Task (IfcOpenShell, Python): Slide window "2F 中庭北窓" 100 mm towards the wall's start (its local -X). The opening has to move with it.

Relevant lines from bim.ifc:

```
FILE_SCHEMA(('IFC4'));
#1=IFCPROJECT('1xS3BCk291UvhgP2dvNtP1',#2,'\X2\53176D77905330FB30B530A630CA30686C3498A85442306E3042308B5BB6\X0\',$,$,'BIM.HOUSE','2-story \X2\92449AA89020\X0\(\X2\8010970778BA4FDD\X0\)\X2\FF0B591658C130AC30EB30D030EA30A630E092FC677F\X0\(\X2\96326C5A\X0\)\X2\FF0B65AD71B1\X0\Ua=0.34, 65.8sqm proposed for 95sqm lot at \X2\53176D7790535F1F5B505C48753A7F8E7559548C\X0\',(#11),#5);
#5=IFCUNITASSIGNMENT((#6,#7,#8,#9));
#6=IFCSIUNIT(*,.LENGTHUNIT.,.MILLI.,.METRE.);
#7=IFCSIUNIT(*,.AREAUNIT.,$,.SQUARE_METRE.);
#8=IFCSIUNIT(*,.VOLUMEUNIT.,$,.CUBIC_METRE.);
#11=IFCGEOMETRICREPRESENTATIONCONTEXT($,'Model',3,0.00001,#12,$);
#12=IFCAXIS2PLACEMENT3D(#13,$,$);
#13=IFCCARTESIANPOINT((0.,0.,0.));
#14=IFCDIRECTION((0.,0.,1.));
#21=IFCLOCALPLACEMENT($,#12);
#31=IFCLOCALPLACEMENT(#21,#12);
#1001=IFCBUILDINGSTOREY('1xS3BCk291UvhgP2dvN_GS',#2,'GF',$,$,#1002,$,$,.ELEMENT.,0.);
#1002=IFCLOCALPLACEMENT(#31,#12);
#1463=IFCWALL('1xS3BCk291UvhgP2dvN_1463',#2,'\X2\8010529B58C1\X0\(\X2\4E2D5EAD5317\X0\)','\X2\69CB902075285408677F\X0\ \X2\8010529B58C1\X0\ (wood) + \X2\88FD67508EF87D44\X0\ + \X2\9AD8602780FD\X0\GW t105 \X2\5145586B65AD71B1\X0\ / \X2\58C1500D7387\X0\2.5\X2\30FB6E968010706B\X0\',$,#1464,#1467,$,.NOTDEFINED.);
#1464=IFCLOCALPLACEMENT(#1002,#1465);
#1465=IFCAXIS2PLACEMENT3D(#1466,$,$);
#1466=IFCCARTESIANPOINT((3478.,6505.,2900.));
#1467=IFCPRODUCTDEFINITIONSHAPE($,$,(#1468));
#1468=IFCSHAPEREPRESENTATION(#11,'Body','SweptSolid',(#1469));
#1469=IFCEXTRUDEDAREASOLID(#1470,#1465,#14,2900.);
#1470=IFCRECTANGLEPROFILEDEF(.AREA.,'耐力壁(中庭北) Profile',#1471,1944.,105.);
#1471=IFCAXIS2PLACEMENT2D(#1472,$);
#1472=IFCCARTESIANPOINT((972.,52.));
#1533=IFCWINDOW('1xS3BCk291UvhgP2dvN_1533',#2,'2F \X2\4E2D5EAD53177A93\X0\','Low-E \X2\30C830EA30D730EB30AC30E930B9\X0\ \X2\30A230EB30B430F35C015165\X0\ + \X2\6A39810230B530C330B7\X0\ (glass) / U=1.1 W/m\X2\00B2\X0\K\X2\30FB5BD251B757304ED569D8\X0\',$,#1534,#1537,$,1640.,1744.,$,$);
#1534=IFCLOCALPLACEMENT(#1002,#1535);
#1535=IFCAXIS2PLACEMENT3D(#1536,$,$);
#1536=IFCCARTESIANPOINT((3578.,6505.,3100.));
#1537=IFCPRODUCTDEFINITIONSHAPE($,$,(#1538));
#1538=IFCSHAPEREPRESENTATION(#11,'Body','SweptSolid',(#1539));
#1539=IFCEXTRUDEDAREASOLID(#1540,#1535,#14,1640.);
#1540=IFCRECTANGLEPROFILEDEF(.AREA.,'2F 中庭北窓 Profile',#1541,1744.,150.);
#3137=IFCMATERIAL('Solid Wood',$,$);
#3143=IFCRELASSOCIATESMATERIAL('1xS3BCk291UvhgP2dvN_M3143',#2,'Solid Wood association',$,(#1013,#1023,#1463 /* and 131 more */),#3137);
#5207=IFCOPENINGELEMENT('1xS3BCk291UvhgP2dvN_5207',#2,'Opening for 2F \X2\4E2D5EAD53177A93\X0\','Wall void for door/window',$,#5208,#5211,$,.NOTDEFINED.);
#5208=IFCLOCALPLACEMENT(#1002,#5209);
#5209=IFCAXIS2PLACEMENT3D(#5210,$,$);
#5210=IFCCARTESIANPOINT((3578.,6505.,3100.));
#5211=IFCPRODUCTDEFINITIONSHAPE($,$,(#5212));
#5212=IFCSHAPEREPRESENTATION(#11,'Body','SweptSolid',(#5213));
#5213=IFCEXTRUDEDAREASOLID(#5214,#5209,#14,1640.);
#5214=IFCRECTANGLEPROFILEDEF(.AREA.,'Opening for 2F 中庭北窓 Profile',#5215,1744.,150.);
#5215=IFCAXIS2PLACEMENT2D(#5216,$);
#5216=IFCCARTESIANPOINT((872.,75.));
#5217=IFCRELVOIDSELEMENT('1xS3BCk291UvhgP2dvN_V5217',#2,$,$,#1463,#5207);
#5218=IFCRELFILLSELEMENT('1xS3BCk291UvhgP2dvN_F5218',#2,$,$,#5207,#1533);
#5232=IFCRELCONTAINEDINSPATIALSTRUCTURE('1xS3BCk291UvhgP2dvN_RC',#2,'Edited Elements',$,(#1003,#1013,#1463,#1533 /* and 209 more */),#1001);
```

```python
import ifcopenshell
import ifcopenshell.api.geometry
import ifcopenshell.util.placement

model = ifcopenshell.open("bim.ifc")

window = model.by_guid("1xS3BCk291UvhgP2dvN_1533")
opening = window.FillsVoids[0].RelatingOpeningElement
wall = opening.VoidsElements[0].RelatingBuildingElement

wall_matrix = ifcopenshell.util.placement.get_local_placement(wall.ObjectPlacement)
shift = wall_matrix[:3, 0] * -100.0
before = ifcopenshell.util.placement.get_local_placement(window.ObjectPlacement)[:3, 3].copy()

# The window is not placed relative to its opening, so move both.
for product in (opening, window):
    matrix = ifcopenshell.util.placement.get_local_placement(product.ObjectPlacement)
    matrix[:3, 3] += shift
    ifcopenshell.api.geometry.edit_object_placement(model, product=product, matrix=matrix, is_si=False)

after = ifcopenshell.util.placement.get_local_placement(window.ObjectPlacement)[:3, 3]
print("window moved by", (after - before).round(3) + 0.0)

model.write("bim_updated.ifc")
```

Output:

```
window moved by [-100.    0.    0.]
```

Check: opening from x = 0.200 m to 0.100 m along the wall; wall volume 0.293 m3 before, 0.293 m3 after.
